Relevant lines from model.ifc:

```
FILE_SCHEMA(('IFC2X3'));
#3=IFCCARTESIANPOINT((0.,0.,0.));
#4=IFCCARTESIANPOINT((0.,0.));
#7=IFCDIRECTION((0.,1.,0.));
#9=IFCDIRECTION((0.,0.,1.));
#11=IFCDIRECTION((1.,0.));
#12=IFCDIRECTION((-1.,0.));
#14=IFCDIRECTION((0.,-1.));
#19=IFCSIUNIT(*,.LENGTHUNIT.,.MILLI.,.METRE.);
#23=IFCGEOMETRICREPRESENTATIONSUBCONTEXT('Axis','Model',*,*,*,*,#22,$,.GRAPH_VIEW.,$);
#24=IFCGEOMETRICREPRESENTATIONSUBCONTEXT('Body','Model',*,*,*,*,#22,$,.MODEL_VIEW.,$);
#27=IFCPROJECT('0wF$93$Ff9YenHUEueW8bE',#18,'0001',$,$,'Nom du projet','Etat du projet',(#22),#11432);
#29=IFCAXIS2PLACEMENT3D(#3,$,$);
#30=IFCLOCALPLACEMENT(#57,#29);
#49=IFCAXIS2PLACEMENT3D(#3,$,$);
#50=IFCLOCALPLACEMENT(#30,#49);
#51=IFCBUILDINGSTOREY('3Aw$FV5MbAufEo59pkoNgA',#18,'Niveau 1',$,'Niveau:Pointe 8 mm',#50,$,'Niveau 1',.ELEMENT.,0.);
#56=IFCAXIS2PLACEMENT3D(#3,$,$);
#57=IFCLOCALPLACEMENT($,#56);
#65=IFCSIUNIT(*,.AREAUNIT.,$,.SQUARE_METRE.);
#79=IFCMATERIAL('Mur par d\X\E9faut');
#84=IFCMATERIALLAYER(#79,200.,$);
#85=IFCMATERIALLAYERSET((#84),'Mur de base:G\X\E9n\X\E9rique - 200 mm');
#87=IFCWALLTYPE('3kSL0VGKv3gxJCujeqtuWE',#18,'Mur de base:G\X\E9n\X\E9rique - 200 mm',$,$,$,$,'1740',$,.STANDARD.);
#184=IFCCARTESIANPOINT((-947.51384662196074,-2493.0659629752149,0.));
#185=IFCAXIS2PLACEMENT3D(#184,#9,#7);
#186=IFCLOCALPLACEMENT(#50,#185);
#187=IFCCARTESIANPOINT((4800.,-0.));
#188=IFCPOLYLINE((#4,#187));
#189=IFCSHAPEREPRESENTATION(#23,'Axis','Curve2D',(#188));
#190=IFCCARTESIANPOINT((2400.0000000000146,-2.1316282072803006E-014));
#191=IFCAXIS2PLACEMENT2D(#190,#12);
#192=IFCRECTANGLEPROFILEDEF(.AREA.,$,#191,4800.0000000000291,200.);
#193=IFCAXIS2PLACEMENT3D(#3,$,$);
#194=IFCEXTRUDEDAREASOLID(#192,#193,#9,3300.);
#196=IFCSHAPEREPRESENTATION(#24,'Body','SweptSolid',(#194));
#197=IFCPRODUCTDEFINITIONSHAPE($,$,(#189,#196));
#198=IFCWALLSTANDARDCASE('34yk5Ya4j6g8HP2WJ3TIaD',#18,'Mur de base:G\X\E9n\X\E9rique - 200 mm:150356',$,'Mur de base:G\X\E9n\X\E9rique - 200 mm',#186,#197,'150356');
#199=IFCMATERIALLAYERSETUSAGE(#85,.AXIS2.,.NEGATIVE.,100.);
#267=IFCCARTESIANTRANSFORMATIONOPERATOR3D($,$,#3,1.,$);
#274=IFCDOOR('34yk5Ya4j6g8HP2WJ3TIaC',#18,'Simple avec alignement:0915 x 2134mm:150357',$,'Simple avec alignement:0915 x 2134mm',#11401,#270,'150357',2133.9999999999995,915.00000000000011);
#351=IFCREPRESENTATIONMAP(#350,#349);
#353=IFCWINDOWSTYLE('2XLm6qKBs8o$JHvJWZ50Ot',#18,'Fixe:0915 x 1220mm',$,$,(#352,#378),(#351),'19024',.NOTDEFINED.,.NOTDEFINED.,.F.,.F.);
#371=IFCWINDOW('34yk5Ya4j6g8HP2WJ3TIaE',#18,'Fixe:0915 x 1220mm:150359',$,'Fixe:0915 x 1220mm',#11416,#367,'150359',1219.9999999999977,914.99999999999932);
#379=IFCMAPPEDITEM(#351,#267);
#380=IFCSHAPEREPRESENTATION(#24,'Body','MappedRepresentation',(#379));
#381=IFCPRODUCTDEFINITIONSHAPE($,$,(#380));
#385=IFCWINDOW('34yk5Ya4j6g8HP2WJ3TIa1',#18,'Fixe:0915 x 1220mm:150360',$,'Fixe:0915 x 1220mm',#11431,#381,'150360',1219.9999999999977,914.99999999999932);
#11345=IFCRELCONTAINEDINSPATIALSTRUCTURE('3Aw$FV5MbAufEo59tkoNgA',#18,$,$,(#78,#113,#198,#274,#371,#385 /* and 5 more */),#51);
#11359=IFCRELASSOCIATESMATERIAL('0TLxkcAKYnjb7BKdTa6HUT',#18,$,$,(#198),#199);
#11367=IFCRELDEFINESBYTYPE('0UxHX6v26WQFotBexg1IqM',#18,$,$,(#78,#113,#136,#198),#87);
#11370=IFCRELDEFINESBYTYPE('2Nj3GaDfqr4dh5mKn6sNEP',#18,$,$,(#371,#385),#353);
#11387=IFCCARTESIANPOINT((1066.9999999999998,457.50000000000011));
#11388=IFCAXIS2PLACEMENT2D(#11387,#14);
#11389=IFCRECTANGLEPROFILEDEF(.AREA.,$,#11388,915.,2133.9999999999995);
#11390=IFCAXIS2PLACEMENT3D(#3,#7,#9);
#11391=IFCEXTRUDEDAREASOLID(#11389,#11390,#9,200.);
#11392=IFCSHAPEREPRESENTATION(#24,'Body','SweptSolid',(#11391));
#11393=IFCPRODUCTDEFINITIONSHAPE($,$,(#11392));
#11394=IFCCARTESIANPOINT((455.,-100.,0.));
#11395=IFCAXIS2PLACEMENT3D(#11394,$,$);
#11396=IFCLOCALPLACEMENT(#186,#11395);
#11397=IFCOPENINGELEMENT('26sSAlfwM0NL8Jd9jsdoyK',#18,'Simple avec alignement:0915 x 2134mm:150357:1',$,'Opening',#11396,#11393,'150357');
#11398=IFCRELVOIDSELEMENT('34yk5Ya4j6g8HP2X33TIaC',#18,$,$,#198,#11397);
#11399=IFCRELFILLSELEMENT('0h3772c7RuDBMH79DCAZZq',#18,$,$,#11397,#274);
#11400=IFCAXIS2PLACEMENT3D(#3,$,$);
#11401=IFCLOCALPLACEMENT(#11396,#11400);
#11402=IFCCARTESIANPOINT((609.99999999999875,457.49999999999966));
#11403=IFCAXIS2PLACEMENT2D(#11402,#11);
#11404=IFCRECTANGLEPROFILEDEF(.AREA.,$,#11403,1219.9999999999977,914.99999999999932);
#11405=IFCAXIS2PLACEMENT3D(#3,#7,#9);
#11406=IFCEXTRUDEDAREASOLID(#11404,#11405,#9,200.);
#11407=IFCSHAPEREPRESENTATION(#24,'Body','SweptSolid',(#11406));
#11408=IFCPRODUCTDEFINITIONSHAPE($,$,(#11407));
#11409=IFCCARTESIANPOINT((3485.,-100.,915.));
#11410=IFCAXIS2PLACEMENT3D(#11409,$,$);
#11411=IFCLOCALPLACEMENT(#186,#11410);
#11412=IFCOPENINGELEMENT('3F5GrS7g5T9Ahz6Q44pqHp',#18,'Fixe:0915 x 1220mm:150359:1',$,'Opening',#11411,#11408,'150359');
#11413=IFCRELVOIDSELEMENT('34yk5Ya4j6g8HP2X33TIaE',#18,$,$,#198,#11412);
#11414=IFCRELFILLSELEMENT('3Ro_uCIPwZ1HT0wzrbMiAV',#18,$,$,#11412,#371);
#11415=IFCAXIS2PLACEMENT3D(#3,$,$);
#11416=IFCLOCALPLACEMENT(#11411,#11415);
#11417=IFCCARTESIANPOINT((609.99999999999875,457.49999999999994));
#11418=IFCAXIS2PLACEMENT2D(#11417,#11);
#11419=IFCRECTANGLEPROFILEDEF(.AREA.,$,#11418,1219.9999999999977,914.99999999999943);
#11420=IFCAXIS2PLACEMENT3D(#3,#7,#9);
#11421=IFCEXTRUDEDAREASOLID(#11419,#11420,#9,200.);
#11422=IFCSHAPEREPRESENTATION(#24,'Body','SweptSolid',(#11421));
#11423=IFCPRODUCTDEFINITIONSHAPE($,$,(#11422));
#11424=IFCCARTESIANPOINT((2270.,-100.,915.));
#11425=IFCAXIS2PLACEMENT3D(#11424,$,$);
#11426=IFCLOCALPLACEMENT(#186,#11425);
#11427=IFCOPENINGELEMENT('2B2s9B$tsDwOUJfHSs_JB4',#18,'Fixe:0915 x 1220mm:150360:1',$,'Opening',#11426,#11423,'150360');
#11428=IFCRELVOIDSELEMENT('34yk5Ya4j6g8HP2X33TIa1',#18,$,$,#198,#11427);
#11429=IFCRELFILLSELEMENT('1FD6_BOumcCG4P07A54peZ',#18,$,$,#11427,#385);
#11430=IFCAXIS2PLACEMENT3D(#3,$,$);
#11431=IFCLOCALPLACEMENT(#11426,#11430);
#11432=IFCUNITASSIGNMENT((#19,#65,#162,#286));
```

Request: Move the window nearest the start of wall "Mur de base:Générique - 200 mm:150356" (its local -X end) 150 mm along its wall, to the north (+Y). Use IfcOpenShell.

```python
import ifcopenshell
import ifcopenshell.api.geometry
import ifcopenshell.util.placement

model = ifcopenshell.open("model.ifc")

window = model.by_id(385)
opening = window.FillsVoids[0].RelatingOpeningElement
wall = opening.VoidsElements[0].RelatingBuildingElement

wall_matrix = ifcopenshell.util.placement.get_local_placement(wall.ObjectPlacement)
shift = wall_matrix[:3, 0] * 150.0
before = ifcopenshell.util.placement.get_local_placement(window.ObjectPlacement)[:3, 3].copy()

# The window is placed relative to its opening, so it follows when the opening moves.
matrix = ifcopenshell.util.placement.get_local_placement(opening.ObjectPlacement)
matrix[:3, 3] += shift
ifcopenshell.api.geometry.edit_object_placement(
    model, product=opening, matrix=matrix, is_si=False, should_transform_children=True
)

after = ifcopenshell.util.placement.get_local_placement(window.ObjectPlacement)[:3, 3]
print("window moved by", (after - before).round(3) + 0.0)

model.write("model_edited.ifc")
```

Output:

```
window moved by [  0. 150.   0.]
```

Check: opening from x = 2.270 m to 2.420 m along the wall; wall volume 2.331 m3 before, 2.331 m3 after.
